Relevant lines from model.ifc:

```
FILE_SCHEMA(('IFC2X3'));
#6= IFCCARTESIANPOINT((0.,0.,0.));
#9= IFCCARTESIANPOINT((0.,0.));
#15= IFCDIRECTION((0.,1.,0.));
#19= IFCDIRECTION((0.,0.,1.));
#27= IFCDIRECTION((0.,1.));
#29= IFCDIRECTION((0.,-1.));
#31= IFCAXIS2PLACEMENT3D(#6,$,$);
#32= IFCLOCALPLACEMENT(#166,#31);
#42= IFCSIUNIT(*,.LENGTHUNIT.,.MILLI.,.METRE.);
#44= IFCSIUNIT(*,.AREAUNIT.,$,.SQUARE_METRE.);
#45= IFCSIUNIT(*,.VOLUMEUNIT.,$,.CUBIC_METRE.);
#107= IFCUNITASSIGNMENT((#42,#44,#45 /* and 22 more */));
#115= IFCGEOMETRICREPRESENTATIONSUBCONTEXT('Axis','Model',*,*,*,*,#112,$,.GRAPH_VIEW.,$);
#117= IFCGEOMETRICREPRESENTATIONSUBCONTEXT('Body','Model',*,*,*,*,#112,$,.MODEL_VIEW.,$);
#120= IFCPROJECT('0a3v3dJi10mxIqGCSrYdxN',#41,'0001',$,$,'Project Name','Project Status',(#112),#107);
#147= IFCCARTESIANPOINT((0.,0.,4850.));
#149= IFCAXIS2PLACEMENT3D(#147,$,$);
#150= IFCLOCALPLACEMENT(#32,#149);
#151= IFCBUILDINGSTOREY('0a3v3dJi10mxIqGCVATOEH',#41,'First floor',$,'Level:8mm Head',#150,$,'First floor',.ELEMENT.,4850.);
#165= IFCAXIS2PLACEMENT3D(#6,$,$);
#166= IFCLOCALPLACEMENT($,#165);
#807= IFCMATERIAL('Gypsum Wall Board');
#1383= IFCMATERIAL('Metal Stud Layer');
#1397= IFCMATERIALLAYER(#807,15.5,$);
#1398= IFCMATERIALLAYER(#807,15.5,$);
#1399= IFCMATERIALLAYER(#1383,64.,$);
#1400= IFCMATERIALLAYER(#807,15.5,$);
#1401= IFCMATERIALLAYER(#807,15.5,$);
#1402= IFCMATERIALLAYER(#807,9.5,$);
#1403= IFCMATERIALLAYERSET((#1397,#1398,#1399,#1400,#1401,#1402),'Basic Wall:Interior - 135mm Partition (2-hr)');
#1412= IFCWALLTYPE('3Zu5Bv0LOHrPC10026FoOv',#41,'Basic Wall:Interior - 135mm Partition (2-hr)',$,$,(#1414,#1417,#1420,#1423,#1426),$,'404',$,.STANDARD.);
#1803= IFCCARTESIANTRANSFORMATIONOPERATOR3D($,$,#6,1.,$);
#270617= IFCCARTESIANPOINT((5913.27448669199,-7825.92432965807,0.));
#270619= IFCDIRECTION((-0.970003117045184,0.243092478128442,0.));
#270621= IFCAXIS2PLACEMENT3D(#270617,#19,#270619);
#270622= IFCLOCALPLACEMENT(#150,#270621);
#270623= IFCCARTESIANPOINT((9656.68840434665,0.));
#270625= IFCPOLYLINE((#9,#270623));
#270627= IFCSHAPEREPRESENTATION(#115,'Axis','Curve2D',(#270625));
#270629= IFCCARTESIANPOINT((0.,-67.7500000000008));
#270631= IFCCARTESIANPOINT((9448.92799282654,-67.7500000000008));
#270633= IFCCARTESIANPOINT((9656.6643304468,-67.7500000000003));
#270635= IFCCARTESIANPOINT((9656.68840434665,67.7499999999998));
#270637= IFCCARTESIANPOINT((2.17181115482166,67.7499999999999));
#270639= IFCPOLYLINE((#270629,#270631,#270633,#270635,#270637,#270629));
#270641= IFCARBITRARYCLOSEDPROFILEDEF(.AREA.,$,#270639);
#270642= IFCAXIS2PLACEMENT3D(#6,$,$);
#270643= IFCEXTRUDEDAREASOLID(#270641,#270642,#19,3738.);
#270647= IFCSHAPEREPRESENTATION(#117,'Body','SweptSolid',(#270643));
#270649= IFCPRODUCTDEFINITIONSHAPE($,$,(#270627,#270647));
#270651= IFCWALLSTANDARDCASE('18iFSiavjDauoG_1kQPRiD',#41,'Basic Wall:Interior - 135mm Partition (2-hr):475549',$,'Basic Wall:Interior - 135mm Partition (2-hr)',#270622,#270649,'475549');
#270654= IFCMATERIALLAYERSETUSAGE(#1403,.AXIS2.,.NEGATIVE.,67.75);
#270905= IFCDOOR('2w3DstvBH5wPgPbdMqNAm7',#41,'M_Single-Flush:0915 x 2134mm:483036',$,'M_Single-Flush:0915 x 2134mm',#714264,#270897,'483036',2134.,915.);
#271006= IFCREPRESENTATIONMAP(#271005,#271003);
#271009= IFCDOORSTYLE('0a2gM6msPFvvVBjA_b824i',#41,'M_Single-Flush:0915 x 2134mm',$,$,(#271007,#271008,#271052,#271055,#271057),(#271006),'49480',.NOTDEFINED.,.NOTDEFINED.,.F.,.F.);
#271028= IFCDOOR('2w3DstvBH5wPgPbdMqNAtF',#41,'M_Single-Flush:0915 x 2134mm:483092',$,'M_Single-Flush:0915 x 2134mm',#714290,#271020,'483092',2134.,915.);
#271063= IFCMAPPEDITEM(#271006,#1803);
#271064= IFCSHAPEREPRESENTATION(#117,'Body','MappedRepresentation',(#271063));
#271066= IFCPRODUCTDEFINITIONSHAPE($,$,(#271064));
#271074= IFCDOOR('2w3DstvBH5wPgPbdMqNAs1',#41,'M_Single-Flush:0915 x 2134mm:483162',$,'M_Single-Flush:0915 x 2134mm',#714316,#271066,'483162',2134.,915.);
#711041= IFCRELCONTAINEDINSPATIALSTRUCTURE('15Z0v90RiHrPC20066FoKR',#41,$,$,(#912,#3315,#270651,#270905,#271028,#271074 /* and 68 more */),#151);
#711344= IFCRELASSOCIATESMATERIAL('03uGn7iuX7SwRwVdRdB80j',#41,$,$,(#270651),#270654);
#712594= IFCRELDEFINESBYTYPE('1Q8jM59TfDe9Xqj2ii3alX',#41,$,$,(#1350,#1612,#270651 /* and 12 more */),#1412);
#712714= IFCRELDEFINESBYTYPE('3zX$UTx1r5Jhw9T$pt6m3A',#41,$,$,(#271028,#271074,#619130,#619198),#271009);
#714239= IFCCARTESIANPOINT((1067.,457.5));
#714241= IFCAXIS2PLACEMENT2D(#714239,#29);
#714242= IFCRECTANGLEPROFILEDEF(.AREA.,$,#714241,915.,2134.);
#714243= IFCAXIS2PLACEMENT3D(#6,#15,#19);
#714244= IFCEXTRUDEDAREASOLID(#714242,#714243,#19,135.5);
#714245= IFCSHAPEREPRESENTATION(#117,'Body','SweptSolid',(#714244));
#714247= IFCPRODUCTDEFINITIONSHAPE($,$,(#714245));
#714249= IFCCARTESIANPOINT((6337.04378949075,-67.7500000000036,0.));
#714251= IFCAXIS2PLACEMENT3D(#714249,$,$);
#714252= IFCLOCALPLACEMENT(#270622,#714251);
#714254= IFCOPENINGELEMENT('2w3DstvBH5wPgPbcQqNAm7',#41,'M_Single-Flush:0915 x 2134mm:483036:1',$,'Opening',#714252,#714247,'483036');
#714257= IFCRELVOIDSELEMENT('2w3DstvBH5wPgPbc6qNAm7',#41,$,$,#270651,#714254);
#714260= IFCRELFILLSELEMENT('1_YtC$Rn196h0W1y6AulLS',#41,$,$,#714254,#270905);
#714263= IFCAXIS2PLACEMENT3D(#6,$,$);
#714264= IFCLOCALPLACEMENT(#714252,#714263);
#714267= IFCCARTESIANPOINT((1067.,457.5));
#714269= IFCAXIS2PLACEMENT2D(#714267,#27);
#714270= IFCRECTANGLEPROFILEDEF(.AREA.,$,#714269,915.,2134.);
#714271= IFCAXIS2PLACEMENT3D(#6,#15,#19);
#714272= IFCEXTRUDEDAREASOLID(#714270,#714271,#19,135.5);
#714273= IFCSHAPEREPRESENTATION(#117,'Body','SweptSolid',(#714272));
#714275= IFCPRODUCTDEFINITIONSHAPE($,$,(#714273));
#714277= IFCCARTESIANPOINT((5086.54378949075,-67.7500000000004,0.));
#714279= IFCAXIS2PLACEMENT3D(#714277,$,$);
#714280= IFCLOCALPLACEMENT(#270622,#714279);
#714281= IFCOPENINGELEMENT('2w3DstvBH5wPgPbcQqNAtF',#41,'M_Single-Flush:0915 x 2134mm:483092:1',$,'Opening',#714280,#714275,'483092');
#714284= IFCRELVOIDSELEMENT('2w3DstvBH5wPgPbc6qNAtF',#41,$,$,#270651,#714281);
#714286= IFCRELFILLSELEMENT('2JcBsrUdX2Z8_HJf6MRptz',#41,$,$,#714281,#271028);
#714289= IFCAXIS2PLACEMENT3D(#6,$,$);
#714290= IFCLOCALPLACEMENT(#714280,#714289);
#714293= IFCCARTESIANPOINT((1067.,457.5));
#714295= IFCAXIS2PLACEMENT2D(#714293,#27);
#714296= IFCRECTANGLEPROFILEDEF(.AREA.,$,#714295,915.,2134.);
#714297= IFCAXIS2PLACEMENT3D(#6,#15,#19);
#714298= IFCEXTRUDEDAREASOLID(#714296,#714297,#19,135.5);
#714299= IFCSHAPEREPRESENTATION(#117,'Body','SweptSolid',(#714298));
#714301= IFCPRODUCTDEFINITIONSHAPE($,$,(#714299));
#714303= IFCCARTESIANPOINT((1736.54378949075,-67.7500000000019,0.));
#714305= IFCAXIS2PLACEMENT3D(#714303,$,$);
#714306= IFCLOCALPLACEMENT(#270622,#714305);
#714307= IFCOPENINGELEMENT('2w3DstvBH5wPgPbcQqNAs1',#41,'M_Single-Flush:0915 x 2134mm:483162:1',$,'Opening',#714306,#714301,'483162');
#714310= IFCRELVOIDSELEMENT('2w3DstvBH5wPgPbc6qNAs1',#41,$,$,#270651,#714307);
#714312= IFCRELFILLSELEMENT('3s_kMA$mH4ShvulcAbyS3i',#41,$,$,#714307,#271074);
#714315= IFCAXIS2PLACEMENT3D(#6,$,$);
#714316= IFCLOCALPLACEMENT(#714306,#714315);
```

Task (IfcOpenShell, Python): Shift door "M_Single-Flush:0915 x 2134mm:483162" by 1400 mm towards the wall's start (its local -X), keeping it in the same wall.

```python
import ifcopenshell
import ifcopenshell.api.geometry
import ifcopenshell.util.placement
import ifcopenshell.util.unit

model = ifcopenshell.open("model.ifc")
unit_scale = ifcopenshell.util.unit.calculate_unit_scale(model)

door = model.by_id(271074)
opening = door.FillsVoids[0].RelatingOpeningElement
wall = opening.VoidsElements[0].RelatingBuildingElement

wall_matrix = ifcopenshell.util.placement.get_local_placement(wall.ObjectPlacement)
shift = wall_matrix[:3, 0] * -1.4 / unit_scale
before = ifcopenshell.util.placement.get_local_placement(door.ObjectPlacement)[:3, 3].copy()

# The door is placed relative to its opening, so it follows when the opening moves.
matrix = ifcopenshell.util.placement.get_local_placement(opening.ObjectPlacement)
matrix[:3, 3] += shift
ifcopenshell.api.geometry.edit_object_placement(
    model, product=opening, matrix=matrix, is_si=False, should_transform_children=True
)

after = ifcopenshell.util.placement.get_local_placement(door.ObjectPlacement)[:3, 3]
print("door moved by", (after - before).round(3) + 0.0)

model.write("model-out.ifc")
```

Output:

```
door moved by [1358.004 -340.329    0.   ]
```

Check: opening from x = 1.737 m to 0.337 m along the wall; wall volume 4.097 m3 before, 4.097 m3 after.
